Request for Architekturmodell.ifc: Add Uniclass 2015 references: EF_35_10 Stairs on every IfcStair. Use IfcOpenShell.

First a look at what the model holds.

```python
import ifcopenshell

model = ifcopenshell.open("Architekturmodell.ifc")
print(model.schema)
print("classifications:", [c.Name for c in model.by_type("IfcClassification")])
for ifc_class in ("IfcDoor", "IfcRoof", "IfcStair", "IfcWall", "IfcWindow"):
    print(ifc_class, len(model.by_type(ifc_class)))
```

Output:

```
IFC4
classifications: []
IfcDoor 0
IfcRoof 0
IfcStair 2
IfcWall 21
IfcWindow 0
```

```python
import ifcopenshell
import ifcopenshell.api.classification

model = ifcopenshell.open("Architekturmodell.ifc")

system = ifcopenshell.api.classification.add_classification(model, classification="Uniclass 2015")

codes = {
    "IfcStair": ("EF_35_10", "Stairs"),
}
for ifc_class, (code, name) in codes.items():
    products = model.by_type(ifc_class)
    ifcopenshell.api.classification.add_reference(
        model, products=products, classification=system, identification=code, name=name
    )
    print(code, len(products))

model.write("Architekturmodell_v2.ifc")
```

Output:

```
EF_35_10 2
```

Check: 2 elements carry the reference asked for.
